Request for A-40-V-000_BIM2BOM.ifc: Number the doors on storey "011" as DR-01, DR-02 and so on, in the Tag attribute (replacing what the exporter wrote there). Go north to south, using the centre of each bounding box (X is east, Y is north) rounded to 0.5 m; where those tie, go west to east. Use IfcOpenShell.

First a look at what the model holds.

```python
import ifcopenshell
import ifcopenshell.util.element
import ifcopenshell.util.placement

model = ifcopenshell.open("A-40-V-000_BIM2BOM.ifc")
print(model.schema)
storey = next(s for s in model.by_type("IfcBuildingStorey") if s.Name == "011")
doors = [e for e in ifcopenshell.util.element.get_decomposition(storey) if e.is_a("IfcDoor")]
for e in sorted(doors, key=lambda e: e.id()):
    origin = ifcopenshell.util.placement.get_local_placement(e.ObjectPlacement)[:3, 3]
    print(e.id(), e.Tag, e.Name, origin.round(2) + 0.0, sep=" | ")
```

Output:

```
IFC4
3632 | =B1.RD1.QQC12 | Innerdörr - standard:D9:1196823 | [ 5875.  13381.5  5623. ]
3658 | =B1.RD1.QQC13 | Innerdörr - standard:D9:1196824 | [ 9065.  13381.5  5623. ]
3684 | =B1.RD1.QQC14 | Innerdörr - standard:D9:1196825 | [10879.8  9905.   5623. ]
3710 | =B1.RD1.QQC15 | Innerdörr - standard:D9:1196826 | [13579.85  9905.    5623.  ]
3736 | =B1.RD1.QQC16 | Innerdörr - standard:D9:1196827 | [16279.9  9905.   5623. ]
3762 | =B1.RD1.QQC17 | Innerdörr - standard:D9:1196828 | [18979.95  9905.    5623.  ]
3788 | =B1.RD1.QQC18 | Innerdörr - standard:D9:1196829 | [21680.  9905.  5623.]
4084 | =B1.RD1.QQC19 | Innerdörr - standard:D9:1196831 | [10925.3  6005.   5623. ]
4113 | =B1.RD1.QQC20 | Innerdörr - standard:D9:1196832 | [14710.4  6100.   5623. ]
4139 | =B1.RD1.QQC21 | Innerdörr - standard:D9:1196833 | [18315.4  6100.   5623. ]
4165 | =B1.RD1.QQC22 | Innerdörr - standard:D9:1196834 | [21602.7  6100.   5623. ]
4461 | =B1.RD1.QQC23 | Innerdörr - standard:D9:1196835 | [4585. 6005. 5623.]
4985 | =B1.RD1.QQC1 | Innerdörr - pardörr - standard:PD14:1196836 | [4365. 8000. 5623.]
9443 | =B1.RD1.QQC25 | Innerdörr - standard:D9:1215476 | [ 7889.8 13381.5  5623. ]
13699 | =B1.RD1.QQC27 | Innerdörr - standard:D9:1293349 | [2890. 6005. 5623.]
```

```python
import ifcopenshell
import ifcopenshell.geom
import ifcopenshell.util.element
import ifcopenshell.util.shape

model = ifcopenshell.open("A-40-V-000_BIM2BOM.ifc")
settings = ifcopenshell.geom.settings()
settings.set("use-world-coords", True)


def centre(element):
    shape = ifcopenshell.geom.create_shape(settings, element)
    return ifcopenshell.util.shape.get_bbox_centroid(shape.geometry)


storey = next(s for s in model.by_type("IfcBuildingStorey") if s.Name == "011")
doors = [e for e in ifcopenshell.util.element.get_decomposition(storey) if e.is_a("IfcDoor")]

# Insertion points can sit at a corner or the storey origin, so sort by the geometry (in metres).
centres = {e: centre(e) for e in doors}
doors.sort(key=lambda e: (-round(centres[e][1] / 0.5), centres[e][0]))

for i, e in enumerate(doors, start=1):
    number = f"DR-{i:02d}"
    e.Tag = number
    print(e.id(), number)

model.write("A-40-V-000_BIM2BOM_v2.ifc")
```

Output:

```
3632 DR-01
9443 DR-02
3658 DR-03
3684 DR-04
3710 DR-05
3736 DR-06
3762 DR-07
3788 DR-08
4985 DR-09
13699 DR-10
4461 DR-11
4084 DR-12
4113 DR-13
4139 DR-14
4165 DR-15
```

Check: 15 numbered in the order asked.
